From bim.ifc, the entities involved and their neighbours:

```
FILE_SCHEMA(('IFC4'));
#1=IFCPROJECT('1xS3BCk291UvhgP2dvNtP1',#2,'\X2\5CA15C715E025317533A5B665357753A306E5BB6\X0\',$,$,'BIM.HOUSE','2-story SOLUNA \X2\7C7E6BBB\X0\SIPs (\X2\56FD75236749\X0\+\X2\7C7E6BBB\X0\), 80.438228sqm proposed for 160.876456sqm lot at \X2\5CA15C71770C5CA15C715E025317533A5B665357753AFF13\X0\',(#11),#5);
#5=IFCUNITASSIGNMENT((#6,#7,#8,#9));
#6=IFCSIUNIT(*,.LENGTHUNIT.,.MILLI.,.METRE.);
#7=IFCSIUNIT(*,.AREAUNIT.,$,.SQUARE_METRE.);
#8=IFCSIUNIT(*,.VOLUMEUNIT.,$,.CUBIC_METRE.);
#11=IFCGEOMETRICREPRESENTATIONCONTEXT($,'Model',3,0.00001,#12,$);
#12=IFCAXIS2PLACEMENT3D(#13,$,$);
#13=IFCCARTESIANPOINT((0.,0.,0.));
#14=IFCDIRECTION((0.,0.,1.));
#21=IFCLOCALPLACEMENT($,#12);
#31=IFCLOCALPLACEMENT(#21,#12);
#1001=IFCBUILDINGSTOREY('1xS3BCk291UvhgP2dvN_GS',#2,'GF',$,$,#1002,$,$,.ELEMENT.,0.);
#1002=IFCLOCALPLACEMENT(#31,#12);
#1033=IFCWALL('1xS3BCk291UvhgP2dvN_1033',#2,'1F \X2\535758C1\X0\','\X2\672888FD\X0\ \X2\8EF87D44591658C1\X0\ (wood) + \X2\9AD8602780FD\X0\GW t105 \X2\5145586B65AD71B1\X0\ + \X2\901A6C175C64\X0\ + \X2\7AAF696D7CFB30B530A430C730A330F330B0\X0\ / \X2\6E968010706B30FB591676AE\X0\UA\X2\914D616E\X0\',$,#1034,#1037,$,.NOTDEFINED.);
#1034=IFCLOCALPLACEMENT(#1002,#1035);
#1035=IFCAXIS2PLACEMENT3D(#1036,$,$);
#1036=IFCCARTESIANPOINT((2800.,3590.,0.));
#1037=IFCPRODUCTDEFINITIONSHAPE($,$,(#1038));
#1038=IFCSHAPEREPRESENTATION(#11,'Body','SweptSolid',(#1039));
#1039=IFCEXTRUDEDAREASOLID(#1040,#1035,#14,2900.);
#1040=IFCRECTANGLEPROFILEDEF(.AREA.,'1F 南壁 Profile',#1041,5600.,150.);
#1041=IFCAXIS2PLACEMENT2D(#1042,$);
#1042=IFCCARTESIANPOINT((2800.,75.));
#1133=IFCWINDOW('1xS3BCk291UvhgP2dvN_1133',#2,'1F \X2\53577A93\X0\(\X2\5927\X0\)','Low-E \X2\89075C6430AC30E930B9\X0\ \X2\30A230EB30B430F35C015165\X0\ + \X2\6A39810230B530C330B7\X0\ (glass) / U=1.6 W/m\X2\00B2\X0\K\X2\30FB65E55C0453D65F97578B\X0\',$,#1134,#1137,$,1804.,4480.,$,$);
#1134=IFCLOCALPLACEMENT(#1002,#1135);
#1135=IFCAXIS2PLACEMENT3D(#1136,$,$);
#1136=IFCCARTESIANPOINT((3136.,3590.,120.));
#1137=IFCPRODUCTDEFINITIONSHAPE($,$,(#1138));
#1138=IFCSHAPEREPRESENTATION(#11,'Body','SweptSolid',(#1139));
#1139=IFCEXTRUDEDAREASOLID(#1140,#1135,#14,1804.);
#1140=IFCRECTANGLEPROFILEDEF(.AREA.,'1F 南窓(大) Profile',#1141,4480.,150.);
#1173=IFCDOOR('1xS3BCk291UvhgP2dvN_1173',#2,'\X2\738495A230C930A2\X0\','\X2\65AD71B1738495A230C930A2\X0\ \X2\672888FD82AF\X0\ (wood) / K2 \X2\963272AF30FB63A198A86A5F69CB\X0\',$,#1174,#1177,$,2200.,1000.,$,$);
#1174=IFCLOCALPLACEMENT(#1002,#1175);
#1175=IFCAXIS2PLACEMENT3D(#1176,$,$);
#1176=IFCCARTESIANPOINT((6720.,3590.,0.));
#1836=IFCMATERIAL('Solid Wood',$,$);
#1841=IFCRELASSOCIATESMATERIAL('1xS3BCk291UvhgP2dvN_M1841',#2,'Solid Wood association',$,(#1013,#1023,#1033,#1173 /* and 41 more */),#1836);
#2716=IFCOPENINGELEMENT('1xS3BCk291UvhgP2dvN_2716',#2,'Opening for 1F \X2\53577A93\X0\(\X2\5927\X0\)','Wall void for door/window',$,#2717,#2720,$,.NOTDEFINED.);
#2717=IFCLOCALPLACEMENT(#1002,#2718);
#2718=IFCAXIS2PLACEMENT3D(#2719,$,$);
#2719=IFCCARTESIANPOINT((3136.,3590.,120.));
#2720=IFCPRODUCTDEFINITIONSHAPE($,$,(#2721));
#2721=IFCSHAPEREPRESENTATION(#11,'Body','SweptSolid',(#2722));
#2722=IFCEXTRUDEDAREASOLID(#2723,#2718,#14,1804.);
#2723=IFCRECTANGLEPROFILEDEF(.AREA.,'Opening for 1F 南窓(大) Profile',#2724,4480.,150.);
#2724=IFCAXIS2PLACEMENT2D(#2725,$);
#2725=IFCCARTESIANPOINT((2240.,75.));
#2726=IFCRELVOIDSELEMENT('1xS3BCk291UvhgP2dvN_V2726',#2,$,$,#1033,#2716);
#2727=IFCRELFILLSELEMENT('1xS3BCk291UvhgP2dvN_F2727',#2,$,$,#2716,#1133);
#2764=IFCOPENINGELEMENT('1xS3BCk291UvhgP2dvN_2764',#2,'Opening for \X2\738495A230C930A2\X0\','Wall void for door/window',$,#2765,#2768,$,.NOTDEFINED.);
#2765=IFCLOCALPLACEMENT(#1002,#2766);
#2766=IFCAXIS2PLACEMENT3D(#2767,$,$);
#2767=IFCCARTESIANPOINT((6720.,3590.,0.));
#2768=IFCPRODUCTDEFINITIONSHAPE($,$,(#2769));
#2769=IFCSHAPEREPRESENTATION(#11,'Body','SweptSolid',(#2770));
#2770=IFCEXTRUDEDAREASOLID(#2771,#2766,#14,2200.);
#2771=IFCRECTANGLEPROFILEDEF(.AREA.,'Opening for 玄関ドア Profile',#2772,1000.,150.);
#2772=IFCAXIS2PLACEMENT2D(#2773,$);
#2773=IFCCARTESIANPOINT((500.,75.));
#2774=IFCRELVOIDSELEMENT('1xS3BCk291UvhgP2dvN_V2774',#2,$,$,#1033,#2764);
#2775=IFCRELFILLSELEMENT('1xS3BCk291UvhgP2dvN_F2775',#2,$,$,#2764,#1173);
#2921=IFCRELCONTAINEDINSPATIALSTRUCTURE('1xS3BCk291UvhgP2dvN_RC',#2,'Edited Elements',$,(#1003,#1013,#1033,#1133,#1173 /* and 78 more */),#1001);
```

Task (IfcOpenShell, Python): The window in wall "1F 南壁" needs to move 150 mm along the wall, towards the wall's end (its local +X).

```python
import ifcopenshell
import ifcopenshell.api.geometry
import ifcopenshell.util.placement

model = ifcopenshell.open("bim.ifc")

window = model.by_guid("1xS3BCk291UvhgP2dvN_1133")
opening = window.FillsVoids[0].RelatingOpeningElement
wall = opening.VoidsElements[0].RelatingBuildingElement

wall_matrix = ifcopenshell.util.placement.get_local_placement(wall.ObjectPlacement)
shift = wall_matrix[:3, 0] * 150.0
before = ifcopenshell.util.placement.get_local_placement(window.ObjectPlacement)[:3, 3].copy()

# The window is not placed relative to its opening, so move both.
for product in (opening, window):
    matrix = ifcopenshell.util.placement.get_local_placement(product.ObjectPlacement)
    matrix[:3, 3] += shift
    ifcopenshell.api.geometry.edit_object_placement(model, product=product, matrix=matrix, is_si=False)

after = ifcopenshell.util.placement.get_local_placement(window.ObjectPlacement)[:3, 3]
print("window moved by", (after - before).round(3) + 0.0)

model.write("bim_v2.ifc")
```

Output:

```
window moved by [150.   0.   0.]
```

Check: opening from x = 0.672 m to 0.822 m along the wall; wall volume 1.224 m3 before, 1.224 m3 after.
